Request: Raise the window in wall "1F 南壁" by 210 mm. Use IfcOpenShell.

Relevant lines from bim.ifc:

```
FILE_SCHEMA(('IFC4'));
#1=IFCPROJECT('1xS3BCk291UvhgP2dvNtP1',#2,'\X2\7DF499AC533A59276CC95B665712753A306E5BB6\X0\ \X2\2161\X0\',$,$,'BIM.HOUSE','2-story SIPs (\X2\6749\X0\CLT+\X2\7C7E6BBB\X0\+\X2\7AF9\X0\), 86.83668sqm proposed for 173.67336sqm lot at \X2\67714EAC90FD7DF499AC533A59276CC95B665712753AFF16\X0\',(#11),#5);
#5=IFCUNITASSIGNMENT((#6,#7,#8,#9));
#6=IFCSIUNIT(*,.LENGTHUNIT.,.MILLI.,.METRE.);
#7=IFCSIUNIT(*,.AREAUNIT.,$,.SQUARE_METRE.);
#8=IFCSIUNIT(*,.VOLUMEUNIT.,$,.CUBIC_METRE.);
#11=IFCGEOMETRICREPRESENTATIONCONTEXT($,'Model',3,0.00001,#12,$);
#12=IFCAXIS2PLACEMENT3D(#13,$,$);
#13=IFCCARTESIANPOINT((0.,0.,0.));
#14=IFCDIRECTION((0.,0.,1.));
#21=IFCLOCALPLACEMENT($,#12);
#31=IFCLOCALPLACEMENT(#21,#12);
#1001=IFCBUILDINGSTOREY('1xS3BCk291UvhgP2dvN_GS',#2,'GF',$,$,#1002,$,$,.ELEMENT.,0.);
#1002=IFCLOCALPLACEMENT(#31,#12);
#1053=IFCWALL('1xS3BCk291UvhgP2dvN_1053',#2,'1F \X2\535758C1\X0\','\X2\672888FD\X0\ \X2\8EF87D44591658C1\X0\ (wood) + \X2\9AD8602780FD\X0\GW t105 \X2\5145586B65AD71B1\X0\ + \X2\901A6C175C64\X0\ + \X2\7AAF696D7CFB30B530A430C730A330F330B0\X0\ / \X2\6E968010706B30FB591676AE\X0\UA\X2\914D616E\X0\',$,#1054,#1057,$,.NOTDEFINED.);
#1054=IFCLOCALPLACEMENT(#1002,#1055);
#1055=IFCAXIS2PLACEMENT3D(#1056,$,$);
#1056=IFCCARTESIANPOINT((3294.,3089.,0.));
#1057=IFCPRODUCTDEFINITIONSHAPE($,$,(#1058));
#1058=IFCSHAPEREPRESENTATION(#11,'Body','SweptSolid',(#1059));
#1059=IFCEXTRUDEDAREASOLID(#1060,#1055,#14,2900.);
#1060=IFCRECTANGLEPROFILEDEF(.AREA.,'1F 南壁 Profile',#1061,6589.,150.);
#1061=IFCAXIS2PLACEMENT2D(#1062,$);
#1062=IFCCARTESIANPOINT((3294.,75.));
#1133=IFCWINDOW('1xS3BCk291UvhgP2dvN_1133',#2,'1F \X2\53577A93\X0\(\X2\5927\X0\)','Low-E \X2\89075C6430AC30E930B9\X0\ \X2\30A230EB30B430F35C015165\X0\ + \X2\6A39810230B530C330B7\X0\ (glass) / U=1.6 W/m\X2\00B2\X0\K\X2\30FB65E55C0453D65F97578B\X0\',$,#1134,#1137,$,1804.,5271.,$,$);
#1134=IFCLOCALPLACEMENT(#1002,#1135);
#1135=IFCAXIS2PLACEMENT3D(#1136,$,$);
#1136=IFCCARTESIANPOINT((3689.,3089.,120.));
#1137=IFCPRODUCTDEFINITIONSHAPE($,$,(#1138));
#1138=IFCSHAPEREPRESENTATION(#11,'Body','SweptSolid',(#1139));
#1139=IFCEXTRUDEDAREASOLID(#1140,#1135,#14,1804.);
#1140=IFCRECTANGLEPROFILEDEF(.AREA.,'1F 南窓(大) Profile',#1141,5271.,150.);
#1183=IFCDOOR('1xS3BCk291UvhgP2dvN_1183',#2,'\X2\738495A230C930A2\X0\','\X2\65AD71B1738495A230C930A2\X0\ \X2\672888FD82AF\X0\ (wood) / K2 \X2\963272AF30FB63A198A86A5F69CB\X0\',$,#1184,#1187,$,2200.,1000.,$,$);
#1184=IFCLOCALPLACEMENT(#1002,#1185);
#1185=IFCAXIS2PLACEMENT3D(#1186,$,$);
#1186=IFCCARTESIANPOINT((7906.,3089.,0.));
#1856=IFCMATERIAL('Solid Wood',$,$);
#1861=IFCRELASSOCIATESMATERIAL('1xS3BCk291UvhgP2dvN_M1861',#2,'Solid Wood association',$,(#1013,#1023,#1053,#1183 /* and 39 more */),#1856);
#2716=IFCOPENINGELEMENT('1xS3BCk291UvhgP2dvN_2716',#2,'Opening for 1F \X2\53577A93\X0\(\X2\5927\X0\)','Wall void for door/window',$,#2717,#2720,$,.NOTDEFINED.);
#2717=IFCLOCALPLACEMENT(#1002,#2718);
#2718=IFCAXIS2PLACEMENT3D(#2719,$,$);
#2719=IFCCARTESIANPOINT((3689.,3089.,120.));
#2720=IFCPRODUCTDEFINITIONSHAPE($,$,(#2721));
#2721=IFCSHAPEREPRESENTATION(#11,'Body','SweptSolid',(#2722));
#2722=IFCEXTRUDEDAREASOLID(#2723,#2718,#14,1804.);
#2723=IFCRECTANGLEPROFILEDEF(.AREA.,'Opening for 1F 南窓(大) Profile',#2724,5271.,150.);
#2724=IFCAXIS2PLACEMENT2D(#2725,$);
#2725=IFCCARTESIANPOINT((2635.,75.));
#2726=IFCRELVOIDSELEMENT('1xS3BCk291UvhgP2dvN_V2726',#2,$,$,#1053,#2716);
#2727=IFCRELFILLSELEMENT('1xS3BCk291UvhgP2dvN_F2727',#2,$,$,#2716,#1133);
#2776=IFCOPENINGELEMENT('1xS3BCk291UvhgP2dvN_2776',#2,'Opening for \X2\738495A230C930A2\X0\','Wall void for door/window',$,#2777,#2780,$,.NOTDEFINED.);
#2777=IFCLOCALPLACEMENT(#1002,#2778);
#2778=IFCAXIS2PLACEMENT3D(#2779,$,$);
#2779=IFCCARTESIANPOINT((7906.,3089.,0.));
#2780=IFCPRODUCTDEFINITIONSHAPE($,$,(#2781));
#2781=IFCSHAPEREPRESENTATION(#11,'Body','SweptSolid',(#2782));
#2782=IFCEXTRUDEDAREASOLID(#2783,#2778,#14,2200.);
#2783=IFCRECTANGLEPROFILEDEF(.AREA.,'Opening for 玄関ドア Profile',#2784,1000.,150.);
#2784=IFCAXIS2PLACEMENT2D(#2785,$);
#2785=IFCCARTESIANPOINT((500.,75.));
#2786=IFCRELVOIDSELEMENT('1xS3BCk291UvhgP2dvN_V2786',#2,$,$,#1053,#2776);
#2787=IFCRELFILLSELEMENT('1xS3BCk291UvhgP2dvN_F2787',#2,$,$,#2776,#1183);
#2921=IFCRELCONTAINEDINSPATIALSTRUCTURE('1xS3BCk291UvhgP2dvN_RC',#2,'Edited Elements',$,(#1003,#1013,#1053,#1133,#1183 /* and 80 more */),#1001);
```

```python
import numpy as np
import ifcopenshell
import ifcopenshell.api.geometry
import ifcopenshell.util.placement
import ifcopenshell.util.unit

model = ifcopenshell.open("bim.ifc")
unit_scale = ifcopenshell.util.unit.calculate_unit_scale(model)

window = model.by_guid("1xS3BCk291UvhgP2dvN_1133")
opening = window.FillsVoids[0].RelatingOpeningElement
dz = 210.0

shift = np.array([0.0, 0.0, dz])
# The window is not placed relative to its opening, so move both.
for product in (opening, window):
    matrix = ifcopenshell.util.placement.get_local_placement(product.ObjectPlacement)
    matrix[:3, 3] += shift
    ifcopenshell.api.geometry.edit_object_placement(model, product=product, matrix=matrix, is_si=False)

print(f"moved by {dz * unit_scale:+.3f} m")

model.write("bim_v2.ifc")
```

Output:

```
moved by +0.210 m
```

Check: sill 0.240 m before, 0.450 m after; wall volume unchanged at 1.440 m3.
